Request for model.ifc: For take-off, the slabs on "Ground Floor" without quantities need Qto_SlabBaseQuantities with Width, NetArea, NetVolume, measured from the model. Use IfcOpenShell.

First a look at what the model holds.

```python
import ifcopenshell
import ifcopenshell.util.element
import ifcopenshell.util.unit

model = ifcopenshell.open("model.ifc")
print(model.schema)
for unit_type in ("LENGTHUNIT", "AREAUNIT", "VOLUMEUNIT"):
    print(unit_type, ifcopenshell.util.unit.calculate_unit_scale(model, unit_type))
storey = next(s for s in model.by_type("IfcBuildingStorey") if s.Name == "Ground Floor")
slabs = [e for e in ifcopenshell.util.element.get_decomposition(storey) if e.is_a("IfcSlab")]
for e in sorted(slabs, key=lambda e: e.id()):
    print(e.id(), e.is_a(), e.Name, list(ifcopenshell.util.element.get_psets(e, qtos_only=True)), sep=" | ")
```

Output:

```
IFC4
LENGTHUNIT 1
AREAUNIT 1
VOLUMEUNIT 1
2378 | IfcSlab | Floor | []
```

```python
import ifcopenshell
import ifcopenshell.api.pset
import ifcopenshell.geom
import ifcopenshell.util.element
import ifcopenshell.util.shape
import ifcopenshell.util.unit

model = ifcopenshell.open("model.ifc")
unit_scale = ifcopenshell.util.unit.calculate_unit_scale(model)
area_scale = ifcopenshell.util.unit.calculate_unit_scale(model, "AREAUNIT")
volume_scale = ifcopenshell.util.unit.calculate_unit_scale(model, "VOLUMEUNIT")
settings = ifcopenshell.geom.settings()

storey = next(s for s in model.by_type("IfcBuildingStorey") if s.Name == "Ground Floor")
slabs = [e for e in ifcopenshell.util.element.get_decomposition(storey) if e.is_a("IfcSlab")]

for e in sorted(slabs, key=lambda e: e.id()):
    if ifcopenshell.util.element.get_psets(e, qtos_only=True, should_inherit=False):
        continue
    # Geometry comes back in metres, in the element's own axes.
    shape = ifcopenshell.geom.create_shape(settings, e)
    values = {
        "Width": ifcopenshell.util.shape.get_z(shape.geometry) / unit_scale,
        "NetArea": ifcopenshell.util.shape.get_footprint_area(shape.geometry) / area_scale,
        "NetVolume": ifcopenshell.util.shape.get_volume(shape.geometry) / volume_scale,
    }
    qto = ifcopenshell.api.pset.add_qto(model, product=e, name="Qto_SlabBaseQuantities")
    ifcopenshell.api.pset.edit_qto(model, qto=qto, properties=values)
    print(e.id(), {k: round(v, 3) for k, v in values.items()})

model.write("model_v2.ifc")
```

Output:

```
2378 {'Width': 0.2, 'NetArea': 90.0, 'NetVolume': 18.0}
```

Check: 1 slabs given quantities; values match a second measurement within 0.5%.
